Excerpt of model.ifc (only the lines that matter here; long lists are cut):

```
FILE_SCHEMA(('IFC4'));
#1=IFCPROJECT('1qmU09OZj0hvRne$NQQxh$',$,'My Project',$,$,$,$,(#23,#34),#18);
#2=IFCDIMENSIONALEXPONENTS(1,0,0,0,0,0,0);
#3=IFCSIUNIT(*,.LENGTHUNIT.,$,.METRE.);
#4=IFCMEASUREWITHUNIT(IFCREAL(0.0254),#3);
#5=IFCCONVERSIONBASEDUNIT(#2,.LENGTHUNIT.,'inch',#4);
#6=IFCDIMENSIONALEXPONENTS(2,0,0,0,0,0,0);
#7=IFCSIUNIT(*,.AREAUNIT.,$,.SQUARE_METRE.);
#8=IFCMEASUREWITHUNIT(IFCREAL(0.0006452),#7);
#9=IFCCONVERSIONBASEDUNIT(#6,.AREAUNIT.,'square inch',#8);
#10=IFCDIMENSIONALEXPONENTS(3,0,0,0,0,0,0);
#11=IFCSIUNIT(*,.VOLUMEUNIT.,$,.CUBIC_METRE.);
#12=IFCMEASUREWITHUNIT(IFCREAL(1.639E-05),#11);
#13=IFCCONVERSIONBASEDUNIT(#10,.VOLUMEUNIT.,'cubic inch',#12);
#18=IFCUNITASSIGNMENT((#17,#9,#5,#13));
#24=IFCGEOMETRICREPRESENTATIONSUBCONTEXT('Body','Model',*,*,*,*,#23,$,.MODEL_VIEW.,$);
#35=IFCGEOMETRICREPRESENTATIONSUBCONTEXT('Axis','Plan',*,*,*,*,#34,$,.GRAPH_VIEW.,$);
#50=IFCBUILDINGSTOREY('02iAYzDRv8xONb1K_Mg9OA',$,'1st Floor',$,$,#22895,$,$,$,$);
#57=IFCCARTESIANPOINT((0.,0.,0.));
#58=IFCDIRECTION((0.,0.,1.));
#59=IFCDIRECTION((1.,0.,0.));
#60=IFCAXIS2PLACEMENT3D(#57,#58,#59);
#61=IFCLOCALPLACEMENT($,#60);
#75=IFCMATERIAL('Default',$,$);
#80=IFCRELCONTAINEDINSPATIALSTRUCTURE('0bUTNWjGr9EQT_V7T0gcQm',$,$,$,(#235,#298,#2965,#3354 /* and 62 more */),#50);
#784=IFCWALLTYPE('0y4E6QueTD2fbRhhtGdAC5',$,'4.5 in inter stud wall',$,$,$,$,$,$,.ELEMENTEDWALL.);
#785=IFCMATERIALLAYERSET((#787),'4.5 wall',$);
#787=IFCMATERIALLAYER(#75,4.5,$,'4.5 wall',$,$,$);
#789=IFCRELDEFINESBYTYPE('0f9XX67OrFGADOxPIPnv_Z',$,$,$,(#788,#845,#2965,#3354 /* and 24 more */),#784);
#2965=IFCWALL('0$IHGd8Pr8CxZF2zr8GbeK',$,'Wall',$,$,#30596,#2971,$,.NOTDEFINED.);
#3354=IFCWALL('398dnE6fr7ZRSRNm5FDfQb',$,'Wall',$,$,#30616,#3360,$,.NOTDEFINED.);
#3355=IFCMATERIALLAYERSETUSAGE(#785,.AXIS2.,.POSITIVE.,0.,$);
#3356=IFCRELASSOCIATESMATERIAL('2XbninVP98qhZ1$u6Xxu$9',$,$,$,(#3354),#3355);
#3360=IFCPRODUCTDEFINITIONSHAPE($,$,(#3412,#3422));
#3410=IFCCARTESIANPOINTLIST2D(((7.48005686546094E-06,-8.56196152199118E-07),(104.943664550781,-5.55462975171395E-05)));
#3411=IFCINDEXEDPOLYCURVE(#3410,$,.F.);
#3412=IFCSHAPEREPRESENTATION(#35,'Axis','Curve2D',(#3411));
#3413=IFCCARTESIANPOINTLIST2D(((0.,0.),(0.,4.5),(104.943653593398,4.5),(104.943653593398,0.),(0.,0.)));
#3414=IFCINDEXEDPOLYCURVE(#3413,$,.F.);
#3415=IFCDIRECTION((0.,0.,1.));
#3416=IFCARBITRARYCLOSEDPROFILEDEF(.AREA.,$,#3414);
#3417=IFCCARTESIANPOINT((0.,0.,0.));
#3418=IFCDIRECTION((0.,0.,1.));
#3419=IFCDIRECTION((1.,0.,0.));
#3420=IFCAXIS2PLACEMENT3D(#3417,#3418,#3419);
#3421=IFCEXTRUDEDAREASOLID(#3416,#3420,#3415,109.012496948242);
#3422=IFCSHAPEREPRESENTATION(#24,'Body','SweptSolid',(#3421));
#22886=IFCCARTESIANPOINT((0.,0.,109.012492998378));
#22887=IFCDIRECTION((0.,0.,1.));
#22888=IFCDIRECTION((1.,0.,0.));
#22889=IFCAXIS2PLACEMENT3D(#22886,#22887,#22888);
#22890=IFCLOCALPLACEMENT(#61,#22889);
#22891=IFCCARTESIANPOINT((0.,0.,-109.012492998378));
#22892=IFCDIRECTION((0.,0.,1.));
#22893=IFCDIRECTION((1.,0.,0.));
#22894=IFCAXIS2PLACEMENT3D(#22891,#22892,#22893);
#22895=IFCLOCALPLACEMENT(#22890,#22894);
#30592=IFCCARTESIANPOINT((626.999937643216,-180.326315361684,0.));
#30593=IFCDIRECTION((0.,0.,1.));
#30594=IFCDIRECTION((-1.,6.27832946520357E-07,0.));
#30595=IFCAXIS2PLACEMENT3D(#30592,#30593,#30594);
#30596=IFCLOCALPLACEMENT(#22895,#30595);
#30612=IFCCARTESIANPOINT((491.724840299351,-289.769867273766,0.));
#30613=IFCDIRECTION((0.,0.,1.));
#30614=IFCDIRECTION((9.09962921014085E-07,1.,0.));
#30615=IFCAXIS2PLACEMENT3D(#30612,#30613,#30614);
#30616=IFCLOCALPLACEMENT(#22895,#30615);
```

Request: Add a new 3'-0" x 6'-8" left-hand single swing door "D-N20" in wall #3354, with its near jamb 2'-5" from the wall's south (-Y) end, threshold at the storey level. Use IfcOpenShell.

```python
import numpy as np
import ifcopenshell
import ifcopenshell.api.feature
import ifcopenshell.api.geometry
import ifcopenshell.api.root
import ifcopenshell.api.spatial
import ifcopenshell.geom
import ifcopenshell.util.element
import ifcopenshell.util.placement
import ifcopenshell.util.representation
import ifcopenshell.util.shape
import ifcopenshell.util.unit

model = ifcopenshell.open("model.ifc")
unit_scale = ifcopenshell.util.unit.calculate_unit_scale(model)
settings = ifcopenshell.geom.settings()


def volume(element):
    """Net volume in cubic metres, openings subtracted."""
    shape = ifcopenshell.geom.create_shape(settings, element)
    return ifcopenshell.util.shape.get_volume(shape.geometry)


wall = model.by_guid("398dnE6fr7ZRSRNm5FDfQb")
storey = ifcopenshell.util.element.get_container(wall, ifc_class="IfcBuildingStorey")
context = ifcopenshell.util.representation.get_context(model, "Model", "Body", "MODEL_VIEW")
before = volume(wall)

width, height, from_end, sill = 0.9144, 2.032, 0.7366, 0.0  # metres

# The wall runs along its own X axis, and the end named is its -X end.
wall_shape = ifcopenshell.geom.create_shape(settings, wall)
x, y, z = ifcopenshell.util.shape.get_vertices(wall_shape.geometry).T
start = x.min() + from_end
face, thickness = float(y.min()), float(y.max() - y.min())
wall_matrix = ifcopenshell.util.placement.get_local_placement(wall.ObjectPlacement)
level = ifcopenshell.util.placement.get_local_placement(storey.ObjectPlacement)[2, 3]


def in_wall(x, y):
    """Placement at x, y metres in the wall's axes, at sill height."""
    matrix = wall_matrix.copy()
    matrix[:, 3] = wall_matrix @ np.array([x / unit_scale, y / unit_scale, 0.0, 1.0])
    matrix[2, 3] = level + sill / unit_scale
    return matrix


# Opening: a box that overshoots both wall faces by 50 mm.
opening = ifcopenshell.api.root.create_entity(model, ifc_class="IfcOpeningElement", predefined_type="OPENING")
box = ifcopenshell.api.geometry.add_wall_representation(
    model, context=context, length=width, height=height, thickness=thickness + 0.1
)
ifcopenshell.api.geometry.assign_representation(model, product=opening, representation=box)
ifcopenshell.api.geometry.edit_object_placement(model, product=opening, matrix=in_wall(start, face - 0.05), is_si=False)
ifcopenshell.api.feature.add_feature(model, feature=opening, element=wall)

door = ifcopenshell.api.root.create_entity(model, ifc_class="IfcDoor", name="D-N20", predefined_type="DOOR")
door.OverallWidth, door.OverallHeight = width / unit_scale, height / unit_scale
door.OperationType = "SINGLE_SWING_LEFT"
body = ifcopenshell.api.geometry.add_door_representation(
    model,
    context=context,
    overall_width=door.OverallWidth,
    overall_height=door.OverallHeight,
    operation_type="SINGLE_SWING_LEFT",
    lining_properties={"LiningDepth": thickness / unit_scale, "ThresholdDepth": thickness / unit_scale},
)
ifcopenshell.api.geometry.assign_representation(model, product=door, representation=body)
ifcopenshell.api.spatial.assign_container(model, products=[door], relating_structure=storey)
ifcopenshell.api.feature.add_filling(model, opening=opening, element=door)

# The lining spans the wall, so the door starts at the wall face.
ifcopenshell.api.geometry.edit_object_placement(model, product=door, matrix=in_wall(start, face), is_si=False)

after = volume(wall)

print(f"wall volume {before:.3f} -> {after:.3f} m3")

model.write("model_v2.ifc")
```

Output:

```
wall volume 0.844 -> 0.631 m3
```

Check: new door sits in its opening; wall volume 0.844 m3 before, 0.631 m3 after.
